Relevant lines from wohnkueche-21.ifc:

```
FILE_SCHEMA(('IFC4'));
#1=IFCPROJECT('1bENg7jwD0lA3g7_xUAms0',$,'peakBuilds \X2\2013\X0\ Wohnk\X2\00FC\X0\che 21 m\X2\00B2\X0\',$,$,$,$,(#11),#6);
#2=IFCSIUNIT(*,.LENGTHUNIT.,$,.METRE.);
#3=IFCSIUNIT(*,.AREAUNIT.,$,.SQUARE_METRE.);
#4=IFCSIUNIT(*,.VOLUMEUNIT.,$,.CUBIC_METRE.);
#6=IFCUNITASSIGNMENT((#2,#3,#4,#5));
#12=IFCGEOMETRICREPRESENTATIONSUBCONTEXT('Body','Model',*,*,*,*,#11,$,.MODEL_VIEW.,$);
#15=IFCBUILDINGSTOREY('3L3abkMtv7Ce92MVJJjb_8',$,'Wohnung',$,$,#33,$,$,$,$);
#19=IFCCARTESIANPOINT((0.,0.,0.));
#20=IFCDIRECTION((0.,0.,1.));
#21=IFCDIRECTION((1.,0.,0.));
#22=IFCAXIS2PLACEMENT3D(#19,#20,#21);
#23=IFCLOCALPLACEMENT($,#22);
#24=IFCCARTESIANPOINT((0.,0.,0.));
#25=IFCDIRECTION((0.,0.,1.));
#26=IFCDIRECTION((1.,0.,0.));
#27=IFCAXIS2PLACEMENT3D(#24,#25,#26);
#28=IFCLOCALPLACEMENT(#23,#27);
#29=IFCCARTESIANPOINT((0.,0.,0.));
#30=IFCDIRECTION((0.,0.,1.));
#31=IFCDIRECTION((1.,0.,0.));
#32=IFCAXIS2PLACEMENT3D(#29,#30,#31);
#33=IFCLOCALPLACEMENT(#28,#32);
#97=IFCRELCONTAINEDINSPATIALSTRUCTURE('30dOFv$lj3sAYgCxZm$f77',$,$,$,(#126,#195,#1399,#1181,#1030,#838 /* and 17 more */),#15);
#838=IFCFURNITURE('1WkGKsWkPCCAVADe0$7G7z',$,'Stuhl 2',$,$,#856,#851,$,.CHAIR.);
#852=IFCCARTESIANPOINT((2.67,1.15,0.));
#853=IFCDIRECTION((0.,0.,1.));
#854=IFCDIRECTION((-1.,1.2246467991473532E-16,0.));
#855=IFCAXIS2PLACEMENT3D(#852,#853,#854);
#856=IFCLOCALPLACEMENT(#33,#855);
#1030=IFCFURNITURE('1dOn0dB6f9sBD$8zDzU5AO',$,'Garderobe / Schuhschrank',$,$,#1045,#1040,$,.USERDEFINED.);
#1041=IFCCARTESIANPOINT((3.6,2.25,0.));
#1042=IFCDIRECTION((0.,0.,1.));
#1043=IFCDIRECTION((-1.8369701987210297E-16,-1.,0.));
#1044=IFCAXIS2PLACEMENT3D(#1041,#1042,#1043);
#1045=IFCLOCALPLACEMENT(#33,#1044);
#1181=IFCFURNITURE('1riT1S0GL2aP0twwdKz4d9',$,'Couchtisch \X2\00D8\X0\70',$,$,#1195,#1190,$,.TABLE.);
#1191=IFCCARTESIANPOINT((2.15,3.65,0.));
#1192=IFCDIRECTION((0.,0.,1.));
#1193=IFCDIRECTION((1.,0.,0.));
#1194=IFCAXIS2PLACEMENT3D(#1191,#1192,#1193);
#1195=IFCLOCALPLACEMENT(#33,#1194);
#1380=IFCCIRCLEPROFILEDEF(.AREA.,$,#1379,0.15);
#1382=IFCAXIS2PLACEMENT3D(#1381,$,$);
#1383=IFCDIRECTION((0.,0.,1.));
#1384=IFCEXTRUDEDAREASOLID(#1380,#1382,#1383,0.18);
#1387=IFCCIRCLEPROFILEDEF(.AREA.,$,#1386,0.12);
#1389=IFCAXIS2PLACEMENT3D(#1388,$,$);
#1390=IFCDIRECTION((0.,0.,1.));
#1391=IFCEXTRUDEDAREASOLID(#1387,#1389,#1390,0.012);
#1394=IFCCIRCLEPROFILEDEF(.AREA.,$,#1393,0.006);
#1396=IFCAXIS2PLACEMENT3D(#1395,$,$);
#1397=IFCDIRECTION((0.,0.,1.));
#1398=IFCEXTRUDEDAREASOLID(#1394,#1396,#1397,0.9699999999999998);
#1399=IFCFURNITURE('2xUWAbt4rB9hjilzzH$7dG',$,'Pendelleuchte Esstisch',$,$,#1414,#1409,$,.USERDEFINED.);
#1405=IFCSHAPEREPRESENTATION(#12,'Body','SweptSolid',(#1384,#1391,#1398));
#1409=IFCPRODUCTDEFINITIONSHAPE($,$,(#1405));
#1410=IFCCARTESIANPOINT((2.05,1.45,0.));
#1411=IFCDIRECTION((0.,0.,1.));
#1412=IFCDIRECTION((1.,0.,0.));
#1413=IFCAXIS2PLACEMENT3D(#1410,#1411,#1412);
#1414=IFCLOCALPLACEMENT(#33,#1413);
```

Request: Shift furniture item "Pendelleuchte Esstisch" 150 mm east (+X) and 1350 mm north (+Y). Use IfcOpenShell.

```python
import ifcopenshell
import ifcopenshell.api.geometry
import ifcopenshell.util.placement
import ifcopenshell.util.unit

model = ifcopenshell.open("wohnkueche-21.ifc")
unit_scale = ifcopenshell.util.unit.calculate_unit_scale(model)

item = model.by_guid("2xUWAbt4rB9hjilzzH$7dG")
matrix = ifcopenshell.util.placement.get_local_placement(item.ObjectPlacement)
matrix[0, 3] += 0.15 / unit_scale
matrix[1, 3] += 1.35 / unit_scale
ifcopenshell.api.geometry.edit_object_placement(model, product=item, matrix=matrix, is_si=False)

print(ifcopenshell.util.placement.get_local_placement(item.ObjectPlacement).round(3) + 0.0)

model.write("wohnkueche-21_v2.ifc")
```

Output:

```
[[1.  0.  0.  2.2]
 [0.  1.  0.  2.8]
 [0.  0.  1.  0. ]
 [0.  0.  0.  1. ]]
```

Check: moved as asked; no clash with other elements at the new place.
